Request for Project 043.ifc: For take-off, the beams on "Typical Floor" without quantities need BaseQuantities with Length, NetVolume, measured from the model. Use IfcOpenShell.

First a look at what the model holds.

```python
import ifcopenshell
import ifcopenshell.util.element
import ifcopenshell.util.unit

model = ifcopenshell.open("Project 043.ifc")
print(model.schema)
for unit_type in ("LENGTHUNIT", "AREAUNIT", "VOLUMEUNIT"):
    print(unit_type, ifcopenshell.util.unit.calculate_unit_scale(model, unit_type))
storey = next(s for s in model.by_type("IfcBuildingStorey") if s.Name == "Typical Floor")
beams = [e for e in ifcopenshell.util.element.get_decomposition(storey) if e.is_a("IfcBeam")]
for e in sorted(beams, key=lambda e: e.id()):
    print(e.id(), e.is_a(), e.Name, list(ifcopenshell.util.element.get_psets(e, qtos_only=True)), sep=" | ")
```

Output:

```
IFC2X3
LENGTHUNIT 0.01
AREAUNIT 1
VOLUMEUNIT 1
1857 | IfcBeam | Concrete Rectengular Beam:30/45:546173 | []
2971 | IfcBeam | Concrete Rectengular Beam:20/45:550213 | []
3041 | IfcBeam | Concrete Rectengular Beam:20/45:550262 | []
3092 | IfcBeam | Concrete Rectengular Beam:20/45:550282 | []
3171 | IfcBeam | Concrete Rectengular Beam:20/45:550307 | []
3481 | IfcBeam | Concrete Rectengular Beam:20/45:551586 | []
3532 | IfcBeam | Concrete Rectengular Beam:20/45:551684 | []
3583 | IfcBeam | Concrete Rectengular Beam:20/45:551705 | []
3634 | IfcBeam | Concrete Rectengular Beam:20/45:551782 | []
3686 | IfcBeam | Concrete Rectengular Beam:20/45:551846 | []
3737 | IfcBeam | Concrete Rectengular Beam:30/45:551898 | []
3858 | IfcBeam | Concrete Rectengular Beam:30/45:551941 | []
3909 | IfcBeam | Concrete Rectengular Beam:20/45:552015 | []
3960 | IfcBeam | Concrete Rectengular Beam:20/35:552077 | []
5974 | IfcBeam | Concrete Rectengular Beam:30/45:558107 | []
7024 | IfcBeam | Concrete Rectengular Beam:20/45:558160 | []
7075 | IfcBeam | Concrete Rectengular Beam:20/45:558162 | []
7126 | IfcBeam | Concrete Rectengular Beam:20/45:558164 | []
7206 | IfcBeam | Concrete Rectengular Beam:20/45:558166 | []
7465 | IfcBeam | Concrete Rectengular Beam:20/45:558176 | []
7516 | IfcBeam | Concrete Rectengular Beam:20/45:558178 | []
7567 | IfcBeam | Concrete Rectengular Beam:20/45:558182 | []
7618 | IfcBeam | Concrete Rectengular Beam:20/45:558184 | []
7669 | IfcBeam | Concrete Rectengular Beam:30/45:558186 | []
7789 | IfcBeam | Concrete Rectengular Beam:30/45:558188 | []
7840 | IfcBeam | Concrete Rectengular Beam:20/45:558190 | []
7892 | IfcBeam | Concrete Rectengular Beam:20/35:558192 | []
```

```python
import ifcopenshell
import ifcopenshell.api.pset
import ifcopenshell.geom
import ifcopenshell.util.element
import ifcopenshell.util.shape
import ifcopenshell.util.unit

model = ifcopenshell.open("Project 043.ifc")
unit_scale = ifcopenshell.util.unit.calculate_unit_scale(model)
volume_scale = ifcopenshell.util.unit.calculate_unit_scale(model, "VOLUMEUNIT")
settings = ifcopenshell.geom.settings()

storey = next(s for s in model.by_type("IfcBuildingStorey") if s.Name == "Typical Floor")
beams = [e for e in ifcopenshell.util.element.get_decomposition(storey) if e.is_a("IfcBeam")]

for e in sorted(beams, key=lambda e: e.id()):
    if ifcopenshell.util.element.get_psets(e, qtos_only=True, should_inherit=False):
        continue
    # Geometry comes back in metres, in the element's own axes.
    shape = ifcopenshell.geom.create_shape(settings, e)
    values = {
        "Length": ifcopenshell.util.shape.get_max_xyz(shape.geometry) / unit_scale,
        "NetVolume": ifcopenshell.util.shape.get_volume(shape.geometry) / volume_scale,
    }
    qto = ifcopenshell.api.pset.add_qto(model, product=e, name="BaseQuantities")
    ifcopenshell.api.pset.edit_qto(model, qto=qto, properties=values)
    print(e.id(), {k: round(v, 3) for k, v in values.items()})

model.write("Project 043_rev.ifc")
```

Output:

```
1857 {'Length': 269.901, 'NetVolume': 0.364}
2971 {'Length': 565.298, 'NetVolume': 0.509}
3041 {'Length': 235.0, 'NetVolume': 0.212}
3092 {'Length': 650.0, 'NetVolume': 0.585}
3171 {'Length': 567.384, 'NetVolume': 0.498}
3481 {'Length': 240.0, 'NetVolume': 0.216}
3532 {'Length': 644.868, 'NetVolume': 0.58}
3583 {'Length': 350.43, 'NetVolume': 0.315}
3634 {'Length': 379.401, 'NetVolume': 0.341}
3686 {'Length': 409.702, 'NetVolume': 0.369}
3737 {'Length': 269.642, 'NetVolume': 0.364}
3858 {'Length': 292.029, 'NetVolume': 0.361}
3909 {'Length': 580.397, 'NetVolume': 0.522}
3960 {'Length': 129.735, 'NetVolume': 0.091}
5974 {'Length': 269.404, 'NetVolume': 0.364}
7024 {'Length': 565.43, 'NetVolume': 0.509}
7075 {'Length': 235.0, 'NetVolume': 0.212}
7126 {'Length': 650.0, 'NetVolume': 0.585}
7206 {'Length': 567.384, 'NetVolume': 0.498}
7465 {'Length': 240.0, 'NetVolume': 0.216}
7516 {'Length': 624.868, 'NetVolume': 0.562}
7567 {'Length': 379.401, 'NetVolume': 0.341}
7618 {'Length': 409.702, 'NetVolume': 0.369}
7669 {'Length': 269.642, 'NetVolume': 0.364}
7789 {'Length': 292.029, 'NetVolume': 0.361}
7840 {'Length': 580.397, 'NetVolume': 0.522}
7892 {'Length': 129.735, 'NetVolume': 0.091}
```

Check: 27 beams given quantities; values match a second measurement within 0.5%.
